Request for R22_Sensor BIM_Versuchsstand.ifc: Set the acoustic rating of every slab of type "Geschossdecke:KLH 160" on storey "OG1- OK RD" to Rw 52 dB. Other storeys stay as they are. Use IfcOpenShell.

First a look at what the model holds.

```python
import ifcopenshell
import ifcopenshell.util.element

model = ifcopenshell.open("R22_Sensor BIM_Versuchsstand.ifc")
print(model.schema)
storey = next(s for s in model.by_type("IfcBuildingStorey") if s.Name == "OG1- OK RD")
slabs = [e for e in ifcopenshell.util.element.get_decomposition(storey) if e.is_a("IfcSlab")]
seen = {}
for e in slabs:
    element_type = ifcopenshell.util.element.get_type(e)
    key = (element_type.Name if element_type != e and element_type else None, ifcopenshell.util.element.get_pset(e, "Pset_SlabCommon", "AcousticRating"))
    seen[key] = seen.get(key, 0) + 1
for (name, value), count in sorted(seen.items(), key=str):
    print(count, "x", name, "|", value)
```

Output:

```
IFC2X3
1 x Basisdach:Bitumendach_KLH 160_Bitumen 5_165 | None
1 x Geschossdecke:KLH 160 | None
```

```python
import ifcopenshell
import ifcopenshell.api.pset
import ifcopenshell.util.element

model = ifcopenshell.open("R22_Sensor BIM_Versuchsstand.ifc")

storey = next(s for s in model.by_type("IfcBuildingStorey") if s.Name == "OG1- OK RD")
slabs = [e for e in ifcopenshell.util.element.get_decomposition(storey) if e.is_a("IfcSlab")]

count = 0
for e in slabs:
    element_type = ifcopenshell.util.element.get_type(e)
    if element_type in (None, e) or element_type.Name != "Geschossdecke:KLH 160":
        continue
    # add_pset returns the element's existing set when there is one.
    pset = ifcopenshell.api.pset.add_pset(model, product=e, name="Pset_SlabCommon")
    ifcopenshell.api.pset.edit_pset(model, pset=pset, properties={"AcousticRating": "Rw 52 dB"})
    count += 1

print(count, "slabs updated")

model.write("R22_Sensor BIM_Versuchsstand_updated.ifc")
```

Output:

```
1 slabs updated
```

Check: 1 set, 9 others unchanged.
